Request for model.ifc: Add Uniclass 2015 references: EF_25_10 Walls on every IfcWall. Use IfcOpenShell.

First a look at what the model holds.

```python
import ifcopenshell

model = ifcopenshell.open("model.ifc")
print(model.schema)
print("classifications:", [c.Name for c in model.by_type("IfcClassification")])
for ifc_class in ("IfcDoor", "IfcRoof", "IfcStair", "IfcWall", "IfcWindow"):
    print(ifc_class, len(model.by_type(ifc_class)))
```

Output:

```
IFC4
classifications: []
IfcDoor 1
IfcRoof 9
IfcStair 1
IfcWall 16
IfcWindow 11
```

```python
import ifcopenshell
import ifcopenshell.api.classification

model = ifcopenshell.open("model.ifc")

system = ifcopenshell.api.classification.add_classification(model, classification="Uniclass 2015")

codes = {
    "IfcWall": ("EF_25_10", "Walls"),
}
for ifc_class, (code, name) in codes.items():
    products = model.by_type(ifc_class)
    ifcopenshell.api.classification.add_reference(
        model, products=products, classification=system, identification=code, name=name
    )
    print(code, len(products))

model.write("model_rev.ifc")
```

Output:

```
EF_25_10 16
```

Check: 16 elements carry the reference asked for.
